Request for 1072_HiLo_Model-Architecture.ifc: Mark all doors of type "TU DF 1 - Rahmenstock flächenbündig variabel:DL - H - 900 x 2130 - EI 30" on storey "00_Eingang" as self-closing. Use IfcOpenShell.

First a look at what the model holds.

```python
import ifcopenshell
import ifcopenshell.util.element

model = ifcopenshell.open("1072_HiLo_Model-Architecture.ifc")
print(model.schema)
storey = next(s for s in model.by_type("IfcBuildingStorey") if s.Name == "00_Eingang")
doors = [e for e in ifcopenshell.util.element.get_decomposition(storey) if e.is_a("IfcDoor")]
seen = {}
for e in doors:
    element_type = ifcopenshell.util.element.get_type(e)
    key = (element_type.Name if element_type != e and element_type else None, ifcopenshell.util.element.get_pset(e, "Pset_DoorCommon", "SelfClosing"))
    seen[key] = seen.get(key, 0) + 1
for (name, value), count in sorted(seen.items(), key=str):
    print(count, "x", name, "|", value)
```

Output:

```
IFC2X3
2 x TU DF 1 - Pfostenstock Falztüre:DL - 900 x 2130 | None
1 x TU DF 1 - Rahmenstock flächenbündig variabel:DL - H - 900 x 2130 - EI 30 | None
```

```python
import ifcopenshell
import ifcopenshell.api.pset
import ifcopenshell.util.element

model = ifcopenshell.open("1072_HiLo_Model-Architecture.ifc")

storey = next(s for s in model.by_type("IfcBuildingStorey") if s.Name == "00_Eingang")
doors = [e for e in ifcopenshell.util.element.get_decomposition(storey) if e.is_a("IfcDoor")]

count = 0
for e in doors:
    element_type = ifcopenshell.util.element.get_type(e)
    if element_type in (None, e) or element_type.Name != "TU DF 1 - Rahmenstock flächenbündig variabel:DL - H - 900 x 2130 - EI 30":
        continue
    # add_pset returns the element's existing set when there is one.
    pset = ifcopenshell.api.pset.add_pset(model, product=e, name="Pset_DoorCommon")
    ifcopenshell.api.pset.edit_pset(model, pset=pset, properties={"SelfClosing": True})
    count += 1

print(count, "doors updated")

model.write("1072_HiLo_Model-Architecture_updated.ifc")
```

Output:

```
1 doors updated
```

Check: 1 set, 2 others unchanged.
